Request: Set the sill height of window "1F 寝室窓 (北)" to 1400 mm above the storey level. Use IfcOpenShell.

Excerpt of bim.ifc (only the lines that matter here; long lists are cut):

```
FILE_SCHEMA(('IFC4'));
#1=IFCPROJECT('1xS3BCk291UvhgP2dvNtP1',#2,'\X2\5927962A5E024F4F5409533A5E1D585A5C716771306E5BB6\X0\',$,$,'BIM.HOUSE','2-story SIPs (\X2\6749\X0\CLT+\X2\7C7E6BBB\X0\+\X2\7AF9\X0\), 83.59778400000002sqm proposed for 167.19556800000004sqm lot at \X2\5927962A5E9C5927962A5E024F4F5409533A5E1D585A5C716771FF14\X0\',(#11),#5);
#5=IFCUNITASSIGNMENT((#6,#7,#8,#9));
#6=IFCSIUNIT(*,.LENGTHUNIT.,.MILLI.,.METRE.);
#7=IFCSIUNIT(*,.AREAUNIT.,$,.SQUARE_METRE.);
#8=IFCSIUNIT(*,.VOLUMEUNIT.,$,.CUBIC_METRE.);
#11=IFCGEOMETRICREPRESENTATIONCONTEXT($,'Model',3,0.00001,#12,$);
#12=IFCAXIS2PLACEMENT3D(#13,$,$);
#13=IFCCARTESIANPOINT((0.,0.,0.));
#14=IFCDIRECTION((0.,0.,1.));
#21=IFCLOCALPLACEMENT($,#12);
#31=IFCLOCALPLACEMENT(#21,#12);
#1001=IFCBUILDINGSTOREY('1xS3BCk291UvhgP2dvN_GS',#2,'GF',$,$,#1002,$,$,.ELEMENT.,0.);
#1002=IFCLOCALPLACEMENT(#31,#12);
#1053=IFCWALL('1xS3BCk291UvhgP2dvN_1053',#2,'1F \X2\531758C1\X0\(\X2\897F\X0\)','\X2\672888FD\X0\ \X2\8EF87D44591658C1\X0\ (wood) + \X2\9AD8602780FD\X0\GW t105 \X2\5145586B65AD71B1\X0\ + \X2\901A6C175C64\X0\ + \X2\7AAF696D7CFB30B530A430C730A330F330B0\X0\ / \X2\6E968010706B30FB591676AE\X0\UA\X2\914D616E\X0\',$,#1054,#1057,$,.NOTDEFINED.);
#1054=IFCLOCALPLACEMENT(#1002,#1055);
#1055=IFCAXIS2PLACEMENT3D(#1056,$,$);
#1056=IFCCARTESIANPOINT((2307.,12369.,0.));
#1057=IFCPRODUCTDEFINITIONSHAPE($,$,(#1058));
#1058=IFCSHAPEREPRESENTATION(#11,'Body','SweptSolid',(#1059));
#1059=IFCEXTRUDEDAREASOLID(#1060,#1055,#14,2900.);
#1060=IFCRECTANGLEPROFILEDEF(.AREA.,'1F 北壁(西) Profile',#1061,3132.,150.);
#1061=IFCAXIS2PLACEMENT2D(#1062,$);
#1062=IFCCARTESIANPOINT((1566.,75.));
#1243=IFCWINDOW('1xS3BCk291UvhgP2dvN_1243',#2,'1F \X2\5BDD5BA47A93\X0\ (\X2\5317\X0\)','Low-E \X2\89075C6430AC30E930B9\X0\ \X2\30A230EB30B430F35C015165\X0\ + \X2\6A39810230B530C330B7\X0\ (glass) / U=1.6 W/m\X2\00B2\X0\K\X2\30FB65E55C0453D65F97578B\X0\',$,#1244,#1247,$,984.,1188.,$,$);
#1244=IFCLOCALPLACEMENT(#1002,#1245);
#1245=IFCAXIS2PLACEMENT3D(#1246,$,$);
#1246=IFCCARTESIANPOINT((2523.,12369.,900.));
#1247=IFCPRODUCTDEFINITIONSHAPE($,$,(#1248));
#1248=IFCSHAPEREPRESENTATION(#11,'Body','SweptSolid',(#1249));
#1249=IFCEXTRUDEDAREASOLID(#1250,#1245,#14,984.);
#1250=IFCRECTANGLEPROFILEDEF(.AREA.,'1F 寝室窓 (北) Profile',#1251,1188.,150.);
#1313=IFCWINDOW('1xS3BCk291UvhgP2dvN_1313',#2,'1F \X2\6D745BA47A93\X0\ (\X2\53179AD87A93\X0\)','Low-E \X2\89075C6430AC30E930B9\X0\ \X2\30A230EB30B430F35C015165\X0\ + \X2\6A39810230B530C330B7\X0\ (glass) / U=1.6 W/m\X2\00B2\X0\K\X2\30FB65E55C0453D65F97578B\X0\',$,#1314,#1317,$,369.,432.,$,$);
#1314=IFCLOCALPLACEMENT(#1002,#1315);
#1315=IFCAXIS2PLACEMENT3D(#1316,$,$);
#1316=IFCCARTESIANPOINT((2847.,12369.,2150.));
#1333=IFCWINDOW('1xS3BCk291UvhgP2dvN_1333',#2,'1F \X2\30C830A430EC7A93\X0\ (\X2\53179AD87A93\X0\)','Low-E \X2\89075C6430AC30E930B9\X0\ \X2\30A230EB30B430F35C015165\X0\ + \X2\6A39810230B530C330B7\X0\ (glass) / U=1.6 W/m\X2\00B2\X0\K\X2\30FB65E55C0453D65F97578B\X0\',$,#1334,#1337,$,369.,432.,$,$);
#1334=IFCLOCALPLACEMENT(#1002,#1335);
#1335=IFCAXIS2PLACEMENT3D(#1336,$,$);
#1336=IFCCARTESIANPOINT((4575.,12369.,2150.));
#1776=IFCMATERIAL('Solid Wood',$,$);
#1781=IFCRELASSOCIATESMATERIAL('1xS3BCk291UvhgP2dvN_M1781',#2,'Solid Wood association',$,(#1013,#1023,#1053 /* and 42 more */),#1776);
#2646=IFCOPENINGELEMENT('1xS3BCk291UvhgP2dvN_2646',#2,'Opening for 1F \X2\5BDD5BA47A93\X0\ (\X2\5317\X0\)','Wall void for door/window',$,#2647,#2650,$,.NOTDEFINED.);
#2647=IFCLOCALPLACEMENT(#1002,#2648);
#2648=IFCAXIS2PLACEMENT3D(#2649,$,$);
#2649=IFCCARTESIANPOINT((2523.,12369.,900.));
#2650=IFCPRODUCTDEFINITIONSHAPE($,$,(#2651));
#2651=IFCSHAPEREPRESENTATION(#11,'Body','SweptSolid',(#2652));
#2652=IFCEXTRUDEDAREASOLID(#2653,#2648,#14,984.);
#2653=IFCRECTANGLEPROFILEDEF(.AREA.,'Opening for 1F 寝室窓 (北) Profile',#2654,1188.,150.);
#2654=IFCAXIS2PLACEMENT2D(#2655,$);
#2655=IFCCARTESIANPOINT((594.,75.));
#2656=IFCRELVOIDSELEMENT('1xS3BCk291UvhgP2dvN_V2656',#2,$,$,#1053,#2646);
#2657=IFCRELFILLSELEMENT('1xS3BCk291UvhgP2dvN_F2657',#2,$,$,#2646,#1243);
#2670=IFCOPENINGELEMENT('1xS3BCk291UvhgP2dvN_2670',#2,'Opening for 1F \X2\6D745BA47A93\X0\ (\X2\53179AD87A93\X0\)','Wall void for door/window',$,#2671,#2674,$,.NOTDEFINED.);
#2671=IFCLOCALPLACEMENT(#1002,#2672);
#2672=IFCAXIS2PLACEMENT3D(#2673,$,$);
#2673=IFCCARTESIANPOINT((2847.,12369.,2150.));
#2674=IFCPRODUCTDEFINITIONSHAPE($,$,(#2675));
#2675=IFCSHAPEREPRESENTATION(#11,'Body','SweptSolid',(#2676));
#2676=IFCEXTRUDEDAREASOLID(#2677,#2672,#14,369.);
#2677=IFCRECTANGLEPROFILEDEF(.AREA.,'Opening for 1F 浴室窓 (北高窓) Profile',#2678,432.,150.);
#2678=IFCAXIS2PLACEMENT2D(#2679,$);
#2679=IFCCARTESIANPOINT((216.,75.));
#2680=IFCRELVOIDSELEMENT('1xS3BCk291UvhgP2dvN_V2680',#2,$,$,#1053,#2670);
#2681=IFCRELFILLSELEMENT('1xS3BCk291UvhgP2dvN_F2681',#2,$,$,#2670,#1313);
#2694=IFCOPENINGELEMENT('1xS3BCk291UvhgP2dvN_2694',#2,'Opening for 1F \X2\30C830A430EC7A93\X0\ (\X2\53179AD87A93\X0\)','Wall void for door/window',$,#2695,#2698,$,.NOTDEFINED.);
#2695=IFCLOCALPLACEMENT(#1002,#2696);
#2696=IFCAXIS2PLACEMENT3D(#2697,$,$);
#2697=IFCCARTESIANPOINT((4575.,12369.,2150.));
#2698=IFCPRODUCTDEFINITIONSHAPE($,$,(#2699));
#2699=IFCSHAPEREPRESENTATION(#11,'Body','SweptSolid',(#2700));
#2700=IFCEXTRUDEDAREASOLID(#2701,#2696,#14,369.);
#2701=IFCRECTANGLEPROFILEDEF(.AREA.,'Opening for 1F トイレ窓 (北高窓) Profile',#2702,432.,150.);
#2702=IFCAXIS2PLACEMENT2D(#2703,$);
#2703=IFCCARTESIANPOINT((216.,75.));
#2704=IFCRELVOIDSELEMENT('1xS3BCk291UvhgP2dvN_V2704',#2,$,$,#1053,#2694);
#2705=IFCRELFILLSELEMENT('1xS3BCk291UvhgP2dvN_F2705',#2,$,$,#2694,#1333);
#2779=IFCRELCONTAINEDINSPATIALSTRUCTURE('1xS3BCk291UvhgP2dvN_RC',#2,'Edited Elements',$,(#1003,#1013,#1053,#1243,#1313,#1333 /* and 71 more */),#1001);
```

```python
import numpy as np
import ifcopenshell
import ifcopenshell.api.geometry
import ifcopenshell.geom
import ifcopenshell.util.element
import ifcopenshell.util.placement
import ifcopenshell.util.shape
import ifcopenshell.util.unit

model = ifcopenshell.open("bim.ifc")
unit_scale = ifcopenshell.util.unit.calculate_unit_scale(model)

window = model.by_guid("1xS3BCk291UvhgP2dvN_1243")
opening = window.FillsVoids[0].RelatingOpeningElement
storey = ifcopenshell.util.element.get_container(window, ifc_class="IfcBuildingStorey")
level = ifcopenshell.util.placement.get_local_placement(storey.ObjectPlacement)[2, 3]

# The opening's origin need not be at the sill, so measure its lowest point.
shape = ifcopenshell.geom.create_shape(ifcopenshell.geom.settings(), opening)
bottom = ifcopenshell.util.shape.get_shape_bottom_elevation(shape, shape.geometry) / unit_scale
dz = level + 1.4 / unit_scale - bottom

shift = np.array([0.0, 0.0, dz])
# The window is not placed relative to its opening, so move both.
for product in (opening, window):
    matrix = ifcopenshell.util.placement.get_local_placement(product.ObjectPlacement)
    matrix[:3, 3] += shift
    ifcopenshell.api.geometry.edit_object_placement(model, product=product, matrix=matrix, is_si=False)

print(f"moved by {dz * unit_scale:+.3f} m")

model.write("bim_updated.ifc")
```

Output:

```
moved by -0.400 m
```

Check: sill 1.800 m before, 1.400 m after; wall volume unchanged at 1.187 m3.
